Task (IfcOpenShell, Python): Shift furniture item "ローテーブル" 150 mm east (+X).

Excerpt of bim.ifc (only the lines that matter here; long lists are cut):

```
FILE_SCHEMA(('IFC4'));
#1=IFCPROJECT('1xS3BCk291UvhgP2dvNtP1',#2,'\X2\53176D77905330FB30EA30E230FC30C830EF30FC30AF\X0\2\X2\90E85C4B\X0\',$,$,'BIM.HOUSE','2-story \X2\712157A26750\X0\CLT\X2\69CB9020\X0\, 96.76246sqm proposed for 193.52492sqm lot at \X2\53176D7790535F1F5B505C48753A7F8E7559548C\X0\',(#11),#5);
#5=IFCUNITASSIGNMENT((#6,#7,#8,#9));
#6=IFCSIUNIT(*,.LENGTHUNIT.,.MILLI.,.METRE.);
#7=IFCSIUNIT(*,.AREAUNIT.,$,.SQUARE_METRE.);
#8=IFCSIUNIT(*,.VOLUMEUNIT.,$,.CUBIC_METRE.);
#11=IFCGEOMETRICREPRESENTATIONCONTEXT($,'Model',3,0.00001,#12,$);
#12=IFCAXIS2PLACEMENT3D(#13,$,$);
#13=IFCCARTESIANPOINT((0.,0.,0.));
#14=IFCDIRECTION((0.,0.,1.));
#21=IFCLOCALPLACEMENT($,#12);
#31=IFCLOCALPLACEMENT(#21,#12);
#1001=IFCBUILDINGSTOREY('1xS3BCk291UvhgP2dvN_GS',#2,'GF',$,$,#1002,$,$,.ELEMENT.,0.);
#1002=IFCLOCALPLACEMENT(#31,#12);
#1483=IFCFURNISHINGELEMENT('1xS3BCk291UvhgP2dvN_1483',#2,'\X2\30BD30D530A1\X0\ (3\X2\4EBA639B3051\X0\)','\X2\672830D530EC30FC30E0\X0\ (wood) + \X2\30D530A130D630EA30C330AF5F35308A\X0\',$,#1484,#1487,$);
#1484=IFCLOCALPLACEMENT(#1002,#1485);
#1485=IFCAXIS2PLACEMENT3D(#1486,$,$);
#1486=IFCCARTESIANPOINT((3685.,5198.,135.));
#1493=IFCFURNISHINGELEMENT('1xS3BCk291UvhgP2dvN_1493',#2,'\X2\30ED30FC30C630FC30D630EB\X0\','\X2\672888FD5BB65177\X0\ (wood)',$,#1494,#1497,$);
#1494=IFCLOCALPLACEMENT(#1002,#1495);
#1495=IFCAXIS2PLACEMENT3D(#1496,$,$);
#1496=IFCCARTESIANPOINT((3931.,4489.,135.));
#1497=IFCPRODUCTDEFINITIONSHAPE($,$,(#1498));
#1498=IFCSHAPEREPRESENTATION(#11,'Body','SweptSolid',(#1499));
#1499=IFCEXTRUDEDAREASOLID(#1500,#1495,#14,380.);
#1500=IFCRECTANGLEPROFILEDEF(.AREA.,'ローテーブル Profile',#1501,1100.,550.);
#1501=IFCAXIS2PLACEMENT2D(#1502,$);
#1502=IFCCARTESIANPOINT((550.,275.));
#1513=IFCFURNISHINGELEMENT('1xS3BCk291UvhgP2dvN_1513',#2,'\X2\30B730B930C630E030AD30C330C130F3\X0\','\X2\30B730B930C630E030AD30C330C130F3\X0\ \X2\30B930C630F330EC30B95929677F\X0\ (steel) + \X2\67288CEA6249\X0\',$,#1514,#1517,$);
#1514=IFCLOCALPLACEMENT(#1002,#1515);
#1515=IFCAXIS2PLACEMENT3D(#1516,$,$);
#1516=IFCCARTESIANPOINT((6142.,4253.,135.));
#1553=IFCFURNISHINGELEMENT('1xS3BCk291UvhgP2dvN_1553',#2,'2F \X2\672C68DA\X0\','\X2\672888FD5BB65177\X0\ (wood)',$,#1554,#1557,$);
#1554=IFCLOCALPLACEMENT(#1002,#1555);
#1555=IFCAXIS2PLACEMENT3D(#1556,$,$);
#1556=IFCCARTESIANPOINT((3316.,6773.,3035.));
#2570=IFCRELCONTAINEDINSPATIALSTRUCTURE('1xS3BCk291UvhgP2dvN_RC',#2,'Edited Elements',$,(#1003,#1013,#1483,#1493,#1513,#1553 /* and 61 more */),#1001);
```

```python
import ifcopenshell
import ifcopenshell.api.geometry
import ifcopenshell.util.placement
import ifcopenshell.util.unit

model = ifcopenshell.open("bim.ifc")
unit_scale = ifcopenshell.util.unit.calculate_unit_scale(model)

item = model.by_id(1493)
matrix = ifcopenshell.util.placement.get_local_placement(item.ObjectPlacement)
matrix[0, 3] += 0.15 / unit_scale
ifcopenshell.api.geometry.edit_object_placement(model, product=item, matrix=matrix, is_si=False)

print(ifcopenshell.util.placement.get_local_placement(item.ObjectPlacement).round(3) + 0.0)

model.write("bim_edited.ifc")
```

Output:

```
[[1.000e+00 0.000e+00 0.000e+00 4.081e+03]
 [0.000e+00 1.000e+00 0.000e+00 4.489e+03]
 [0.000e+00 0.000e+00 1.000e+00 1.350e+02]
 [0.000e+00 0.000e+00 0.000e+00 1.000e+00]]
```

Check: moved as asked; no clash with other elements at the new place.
